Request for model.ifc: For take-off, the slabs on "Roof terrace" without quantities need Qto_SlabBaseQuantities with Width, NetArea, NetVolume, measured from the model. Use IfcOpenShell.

First a look at what the model holds.

```python
import ifcopenshell
import ifcopenshell.util.element
import ifcopenshell.util.unit

model = ifcopenshell.open("model.ifc")
print(model.schema)
for unit_type in ("LENGTHUNIT", "AREAUNIT", "VOLUMEUNIT"):
    print(unit_type, ifcopenshell.util.unit.calculate_unit_scale(model, unit_type))
storey = next(s for s in model.by_type("IfcBuildingStorey") if s.Name == "Roof terrace")
slabs = [e for e in ifcopenshell.util.element.get_decomposition(storey) if e.is_a("IfcSlab")]
for e in sorted(slabs, key=lambda e: e.id()):
    print(e.id(), e.is_a(), e.Name, list(ifcopenshell.util.element.get_psets(e, qtos_only=True)), sep=" | ")
```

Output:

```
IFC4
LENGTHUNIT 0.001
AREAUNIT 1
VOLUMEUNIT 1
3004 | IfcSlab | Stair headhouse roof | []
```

```python
import ifcopenshell
import ifcopenshell.api.pset
import ifcopenshell.geom
import ifcopenshell.util.element
import ifcopenshell.util.shape
import ifcopenshell.util.unit

model = ifcopenshell.open("model.ifc")
unit_scale = ifcopenshell.util.unit.calculate_unit_scale(model)
area_scale = ifcopenshell.util.unit.calculate_unit_scale(model, "AREAUNIT")
volume_scale = ifcopenshell.util.unit.calculate_unit_scale(model, "VOLUMEUNIT")
settings = ifcopenshell.geom.settings()

storey = next(s for s in model.by_type("IfcBuildingStorey") if s.Name == "Roof terrace")
slabs = [e for e in ifcopenshell.util.element.get_decomposition(storey) if e.is_a("IfcSlab")]

for e in sorted(slabs, key=lambda e: e.id()):
    if ifcopenshell.util.element.get_psets(e, qtos_only=True, should_inherit=False):
        continue
    # Geometry comes back in metres, in the element's own axes.
    shape = ifcopenshell.geom.create_shape(settings, e)
    values = {
        "Width": ifcopenshell.util.shape.get_z(shape.geometry) / unit_scale,
        "NetArea": ifcopenshell.util.shape.get_footprint_area(shape.geometry) / area_scale,
        "NetVolume": ifcopenshell.util.shape.get_volume(shape.geometry) / volume_scale,
    }
    qto = ifcopenshell.api.pset.add_qto(model, product=e, name="Qto_SlabBaseQuantities")
    ifcopenshell.api.pset.edit_qto(model, qto=qto, properties=values)
    print(e.id(), {k: round(v, 3) for k, v in values.items()})

model.write("model-out.ifc")
```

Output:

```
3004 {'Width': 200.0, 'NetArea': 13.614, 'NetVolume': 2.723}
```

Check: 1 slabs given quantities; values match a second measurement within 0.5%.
